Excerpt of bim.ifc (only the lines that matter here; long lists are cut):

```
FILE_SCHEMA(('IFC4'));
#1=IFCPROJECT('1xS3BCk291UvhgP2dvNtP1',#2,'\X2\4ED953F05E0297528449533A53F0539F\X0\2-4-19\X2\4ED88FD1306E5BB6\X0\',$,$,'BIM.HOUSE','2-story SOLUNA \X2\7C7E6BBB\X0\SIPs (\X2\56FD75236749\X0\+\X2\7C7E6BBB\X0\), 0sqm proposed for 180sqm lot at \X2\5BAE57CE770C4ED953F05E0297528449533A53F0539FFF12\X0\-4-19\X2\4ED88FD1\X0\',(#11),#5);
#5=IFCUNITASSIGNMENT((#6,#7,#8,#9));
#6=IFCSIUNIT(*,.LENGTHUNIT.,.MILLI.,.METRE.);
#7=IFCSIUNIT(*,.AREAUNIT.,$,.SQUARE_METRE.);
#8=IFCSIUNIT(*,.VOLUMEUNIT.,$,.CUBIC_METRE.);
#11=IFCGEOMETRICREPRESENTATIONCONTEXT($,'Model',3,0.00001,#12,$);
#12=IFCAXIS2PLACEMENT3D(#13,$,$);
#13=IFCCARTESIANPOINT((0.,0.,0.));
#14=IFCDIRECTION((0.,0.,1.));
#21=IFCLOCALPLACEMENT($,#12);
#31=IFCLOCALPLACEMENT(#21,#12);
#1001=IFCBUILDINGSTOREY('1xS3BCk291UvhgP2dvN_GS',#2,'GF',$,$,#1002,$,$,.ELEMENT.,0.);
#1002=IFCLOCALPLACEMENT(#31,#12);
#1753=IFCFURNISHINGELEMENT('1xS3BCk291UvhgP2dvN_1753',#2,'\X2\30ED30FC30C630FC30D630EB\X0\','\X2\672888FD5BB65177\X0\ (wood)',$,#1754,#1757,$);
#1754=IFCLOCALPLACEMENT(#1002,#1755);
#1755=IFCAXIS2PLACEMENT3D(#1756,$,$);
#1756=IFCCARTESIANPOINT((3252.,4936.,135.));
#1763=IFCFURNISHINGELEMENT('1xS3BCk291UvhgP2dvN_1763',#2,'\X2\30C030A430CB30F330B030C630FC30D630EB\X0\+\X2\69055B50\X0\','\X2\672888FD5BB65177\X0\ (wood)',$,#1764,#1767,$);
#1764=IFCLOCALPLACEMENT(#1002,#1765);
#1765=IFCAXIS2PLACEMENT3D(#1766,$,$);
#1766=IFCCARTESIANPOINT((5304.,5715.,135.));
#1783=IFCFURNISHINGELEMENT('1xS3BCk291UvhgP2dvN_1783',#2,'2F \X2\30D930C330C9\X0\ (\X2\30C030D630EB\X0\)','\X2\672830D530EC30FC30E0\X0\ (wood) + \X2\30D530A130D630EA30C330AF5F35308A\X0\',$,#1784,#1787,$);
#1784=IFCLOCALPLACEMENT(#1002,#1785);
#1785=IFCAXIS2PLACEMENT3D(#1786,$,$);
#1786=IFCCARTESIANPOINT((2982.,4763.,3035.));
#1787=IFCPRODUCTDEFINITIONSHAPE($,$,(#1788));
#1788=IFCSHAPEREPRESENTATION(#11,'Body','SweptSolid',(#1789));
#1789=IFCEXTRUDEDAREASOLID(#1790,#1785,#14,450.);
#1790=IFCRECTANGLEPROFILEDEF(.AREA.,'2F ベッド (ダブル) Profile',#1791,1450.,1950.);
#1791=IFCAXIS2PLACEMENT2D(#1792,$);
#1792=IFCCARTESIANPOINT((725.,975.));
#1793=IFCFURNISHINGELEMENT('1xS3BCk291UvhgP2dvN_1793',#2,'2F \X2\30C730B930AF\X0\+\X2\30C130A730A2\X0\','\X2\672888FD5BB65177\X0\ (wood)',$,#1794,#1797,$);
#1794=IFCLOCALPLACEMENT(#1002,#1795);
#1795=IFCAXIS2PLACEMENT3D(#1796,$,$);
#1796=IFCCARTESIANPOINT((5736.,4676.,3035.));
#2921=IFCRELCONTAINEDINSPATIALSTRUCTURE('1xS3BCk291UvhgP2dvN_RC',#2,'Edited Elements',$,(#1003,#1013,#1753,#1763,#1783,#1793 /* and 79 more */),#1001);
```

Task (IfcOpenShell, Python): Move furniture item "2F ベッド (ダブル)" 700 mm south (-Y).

```python
import ifcopenshell
import ifcopenshell.api.geometry
import ifcopenshell.util.placement

model = ifcopenshell.open("bim.ifc")

item = model.by_guid("1xS3BCk291UvhgP2dvN_1783")
matrix = ifcopenshell.util.placement.get_local_placement(item.ObjectPlacement)
matrix[1, 3] -= 700.0
ifcopenshell.api.geometry.edit_object_placement(model, product=item, matrix=matrix, is_si=False)

print(ifcopenshell.util.placement.get_local_placement(item.ObjectPlacement).round(3) + 0.0)

model.write("bim-out.ifc")
```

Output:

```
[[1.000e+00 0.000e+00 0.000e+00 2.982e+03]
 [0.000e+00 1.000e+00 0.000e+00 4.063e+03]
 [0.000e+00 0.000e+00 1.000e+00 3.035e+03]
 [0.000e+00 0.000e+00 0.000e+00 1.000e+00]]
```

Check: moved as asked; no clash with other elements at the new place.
